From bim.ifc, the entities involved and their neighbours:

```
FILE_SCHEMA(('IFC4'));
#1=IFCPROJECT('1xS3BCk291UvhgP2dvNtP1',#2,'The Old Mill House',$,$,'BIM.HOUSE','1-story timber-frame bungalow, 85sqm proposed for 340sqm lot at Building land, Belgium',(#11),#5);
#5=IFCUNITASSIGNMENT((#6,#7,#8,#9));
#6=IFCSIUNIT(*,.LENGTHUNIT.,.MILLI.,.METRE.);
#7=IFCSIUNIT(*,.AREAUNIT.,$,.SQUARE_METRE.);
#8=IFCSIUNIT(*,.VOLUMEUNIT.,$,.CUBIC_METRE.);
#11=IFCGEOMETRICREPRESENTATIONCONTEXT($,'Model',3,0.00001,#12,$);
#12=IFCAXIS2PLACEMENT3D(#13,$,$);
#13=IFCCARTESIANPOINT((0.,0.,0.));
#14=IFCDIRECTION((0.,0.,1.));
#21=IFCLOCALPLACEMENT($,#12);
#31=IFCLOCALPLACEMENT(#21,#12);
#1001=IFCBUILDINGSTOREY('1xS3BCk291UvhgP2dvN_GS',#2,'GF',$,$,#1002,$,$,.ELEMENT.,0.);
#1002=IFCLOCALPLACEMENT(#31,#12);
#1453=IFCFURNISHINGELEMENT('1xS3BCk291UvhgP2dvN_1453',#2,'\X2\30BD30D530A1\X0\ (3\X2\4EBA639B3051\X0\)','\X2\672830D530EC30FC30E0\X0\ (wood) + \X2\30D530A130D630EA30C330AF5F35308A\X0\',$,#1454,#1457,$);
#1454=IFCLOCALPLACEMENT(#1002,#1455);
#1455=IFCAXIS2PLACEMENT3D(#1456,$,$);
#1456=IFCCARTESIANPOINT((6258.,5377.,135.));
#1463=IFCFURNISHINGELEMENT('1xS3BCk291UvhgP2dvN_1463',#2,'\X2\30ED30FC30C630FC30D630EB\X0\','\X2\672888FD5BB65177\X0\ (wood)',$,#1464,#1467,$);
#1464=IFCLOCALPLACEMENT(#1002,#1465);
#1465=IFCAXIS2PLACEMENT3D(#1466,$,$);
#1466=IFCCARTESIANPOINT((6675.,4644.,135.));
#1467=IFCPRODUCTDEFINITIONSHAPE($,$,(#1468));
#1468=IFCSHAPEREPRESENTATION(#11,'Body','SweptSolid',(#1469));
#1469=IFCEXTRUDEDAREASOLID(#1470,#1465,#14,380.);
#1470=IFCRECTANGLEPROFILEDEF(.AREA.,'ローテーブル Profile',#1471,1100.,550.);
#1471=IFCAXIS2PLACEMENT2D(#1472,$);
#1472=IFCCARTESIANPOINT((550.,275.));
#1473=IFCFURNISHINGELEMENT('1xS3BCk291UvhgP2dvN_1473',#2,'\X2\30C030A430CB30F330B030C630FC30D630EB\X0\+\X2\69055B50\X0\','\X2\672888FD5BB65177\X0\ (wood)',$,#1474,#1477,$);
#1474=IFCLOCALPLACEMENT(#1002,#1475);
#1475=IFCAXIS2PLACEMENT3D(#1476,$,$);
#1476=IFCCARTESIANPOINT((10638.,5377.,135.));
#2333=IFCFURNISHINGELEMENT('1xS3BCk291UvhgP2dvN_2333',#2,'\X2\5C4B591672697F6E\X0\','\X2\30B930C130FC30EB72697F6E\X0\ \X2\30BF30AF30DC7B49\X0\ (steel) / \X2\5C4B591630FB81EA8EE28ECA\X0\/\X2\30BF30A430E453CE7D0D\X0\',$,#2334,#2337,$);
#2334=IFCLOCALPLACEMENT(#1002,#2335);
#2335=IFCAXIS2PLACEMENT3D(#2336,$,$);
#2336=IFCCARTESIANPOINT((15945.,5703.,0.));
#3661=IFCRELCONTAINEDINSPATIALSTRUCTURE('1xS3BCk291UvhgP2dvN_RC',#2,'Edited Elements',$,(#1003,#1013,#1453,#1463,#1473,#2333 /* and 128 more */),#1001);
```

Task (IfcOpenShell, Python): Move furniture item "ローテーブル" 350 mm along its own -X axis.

```python
import ifcopenshell
import ifcopenshell.api.geometry
import ifcopenshell.util.placement
import ifcopenshell.util.unit

model = ifcopenshell.open("bim.ifc")
unit_scale = ifcopenshell.util.unit.calculate_unit_scale(model)

item = model.by_guid("1xS3BCk291UvhgP2dvN_1463")
matrix = ifcopenshell.util.placement.get_local_placement(item.ObjectPlacement)
matrix[:3, 3] -= matrix[:3, 0] * 0.35 / unit_scale
ifcopenshell.api.geometry.edit_object_placement(model, product=item, matrix=matrix, is_si=False)

print(ifcopenshell.util.placement.get_local_placement(item.ObjectPlacement).round(3) + 0.0)

model.write("bim_v2.ifc")
```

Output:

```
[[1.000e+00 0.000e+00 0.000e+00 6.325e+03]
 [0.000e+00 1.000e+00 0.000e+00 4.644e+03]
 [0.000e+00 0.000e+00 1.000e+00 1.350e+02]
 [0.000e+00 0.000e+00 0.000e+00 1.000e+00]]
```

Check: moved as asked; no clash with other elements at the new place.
